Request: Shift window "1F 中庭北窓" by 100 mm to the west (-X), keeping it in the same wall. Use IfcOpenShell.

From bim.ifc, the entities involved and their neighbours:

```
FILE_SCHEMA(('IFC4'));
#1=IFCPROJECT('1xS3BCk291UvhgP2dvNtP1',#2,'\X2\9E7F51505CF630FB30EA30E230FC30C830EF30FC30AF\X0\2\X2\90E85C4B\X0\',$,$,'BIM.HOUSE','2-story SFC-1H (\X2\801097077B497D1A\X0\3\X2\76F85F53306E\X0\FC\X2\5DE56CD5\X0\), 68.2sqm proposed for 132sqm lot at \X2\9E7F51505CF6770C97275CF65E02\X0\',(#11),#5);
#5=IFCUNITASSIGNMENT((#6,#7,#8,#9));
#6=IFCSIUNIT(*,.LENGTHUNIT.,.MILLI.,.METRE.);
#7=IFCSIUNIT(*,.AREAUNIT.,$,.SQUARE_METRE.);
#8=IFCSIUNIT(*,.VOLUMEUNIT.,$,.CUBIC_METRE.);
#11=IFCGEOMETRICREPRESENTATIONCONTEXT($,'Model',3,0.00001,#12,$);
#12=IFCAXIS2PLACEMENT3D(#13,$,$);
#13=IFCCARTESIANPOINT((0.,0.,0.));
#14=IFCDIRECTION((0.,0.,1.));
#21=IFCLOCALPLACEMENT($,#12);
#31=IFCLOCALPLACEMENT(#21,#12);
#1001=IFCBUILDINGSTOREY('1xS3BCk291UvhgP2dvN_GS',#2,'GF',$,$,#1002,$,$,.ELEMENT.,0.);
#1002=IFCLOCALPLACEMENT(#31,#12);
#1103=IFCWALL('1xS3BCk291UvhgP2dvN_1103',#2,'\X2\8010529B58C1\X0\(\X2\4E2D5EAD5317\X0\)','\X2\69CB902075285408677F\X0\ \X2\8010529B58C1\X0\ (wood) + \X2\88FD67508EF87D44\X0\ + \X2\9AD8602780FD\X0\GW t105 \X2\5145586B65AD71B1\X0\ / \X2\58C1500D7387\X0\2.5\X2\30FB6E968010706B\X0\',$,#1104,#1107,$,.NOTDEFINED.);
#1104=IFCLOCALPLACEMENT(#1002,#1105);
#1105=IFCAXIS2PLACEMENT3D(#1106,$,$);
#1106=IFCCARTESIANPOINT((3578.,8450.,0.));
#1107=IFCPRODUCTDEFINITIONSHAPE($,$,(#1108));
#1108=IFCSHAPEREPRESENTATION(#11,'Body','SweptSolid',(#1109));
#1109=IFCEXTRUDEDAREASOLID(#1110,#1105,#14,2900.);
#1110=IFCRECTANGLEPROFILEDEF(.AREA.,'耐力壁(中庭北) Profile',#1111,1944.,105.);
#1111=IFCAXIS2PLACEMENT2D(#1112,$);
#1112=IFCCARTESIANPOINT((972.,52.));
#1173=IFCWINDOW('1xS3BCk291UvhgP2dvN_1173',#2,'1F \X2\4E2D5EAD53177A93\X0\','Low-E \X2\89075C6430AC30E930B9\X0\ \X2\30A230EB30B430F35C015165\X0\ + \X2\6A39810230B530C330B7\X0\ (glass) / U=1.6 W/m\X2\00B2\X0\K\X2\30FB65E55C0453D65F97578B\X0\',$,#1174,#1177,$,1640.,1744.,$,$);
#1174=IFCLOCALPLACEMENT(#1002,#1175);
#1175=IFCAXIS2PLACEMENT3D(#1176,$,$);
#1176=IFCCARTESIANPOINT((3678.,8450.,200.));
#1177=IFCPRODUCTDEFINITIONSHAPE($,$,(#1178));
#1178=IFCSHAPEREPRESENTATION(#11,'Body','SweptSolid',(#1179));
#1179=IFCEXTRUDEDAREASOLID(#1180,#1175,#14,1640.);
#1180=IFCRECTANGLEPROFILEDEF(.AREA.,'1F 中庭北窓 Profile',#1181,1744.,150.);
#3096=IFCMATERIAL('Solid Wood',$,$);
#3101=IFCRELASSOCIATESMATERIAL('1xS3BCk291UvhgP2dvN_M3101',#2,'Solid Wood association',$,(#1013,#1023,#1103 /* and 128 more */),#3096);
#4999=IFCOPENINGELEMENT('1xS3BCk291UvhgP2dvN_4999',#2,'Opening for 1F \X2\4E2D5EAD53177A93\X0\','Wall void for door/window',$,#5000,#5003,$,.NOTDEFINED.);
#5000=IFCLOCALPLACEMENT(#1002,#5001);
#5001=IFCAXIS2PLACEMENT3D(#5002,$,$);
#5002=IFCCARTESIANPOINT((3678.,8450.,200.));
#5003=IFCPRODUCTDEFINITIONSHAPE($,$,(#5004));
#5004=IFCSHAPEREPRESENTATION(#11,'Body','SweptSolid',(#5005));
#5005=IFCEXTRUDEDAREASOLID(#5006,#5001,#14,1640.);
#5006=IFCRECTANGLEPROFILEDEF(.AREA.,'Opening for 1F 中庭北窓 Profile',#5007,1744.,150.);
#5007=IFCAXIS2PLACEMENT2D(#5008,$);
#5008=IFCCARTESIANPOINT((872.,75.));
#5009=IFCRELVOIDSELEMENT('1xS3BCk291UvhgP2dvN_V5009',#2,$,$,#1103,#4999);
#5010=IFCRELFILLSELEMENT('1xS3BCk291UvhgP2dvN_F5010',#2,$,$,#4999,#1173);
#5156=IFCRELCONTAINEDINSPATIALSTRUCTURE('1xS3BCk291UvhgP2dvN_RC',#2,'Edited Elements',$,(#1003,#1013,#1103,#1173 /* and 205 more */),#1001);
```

```python
import ifcopenshell
import ifcopenshell.api.geometry
import ifcopenshell.util.placement
import ifcopenshell.util.unit

model = ifcopenshell.open("bim.ifc")
unit_scale = ifcopenshell.util.unit.calculate_unit_scale(model)

window = model.by_id(1173)
opening = window.FillsVoids[0].RelatingOpeningElement
wall = opening.VoidsElements[0].RelatingBuildingElement

wall_matrix = ifcopenshell.util.placement.get_local_placement(wall.ObjectPlacement)
shift = wall_matrix[:3, 0] * -0.1 / unit_scale
before = ifcopenshell.util.placement.get_local_placement(window.ObjectPlacement)[:3, 3].copy()

# The window is not placed relative to its opening, so move both.
for product in (opening, window):
    matrix = ifcopenshell.util.placement.get_local_placement(product.ObjectPlacement)
    matrix[:3, 3] += shift
    ifcopenshell.api.geometry.edit_object_placement(model, product=product, matrix=matrix, is_si=False)

after = ifcopenshell.util.placement.get_local_placement(window.ObjectPlacement)[:3, 3]
print("window moved by", (after - before).round(3) + 0.0)

model.write("bim_v2.ifc")
```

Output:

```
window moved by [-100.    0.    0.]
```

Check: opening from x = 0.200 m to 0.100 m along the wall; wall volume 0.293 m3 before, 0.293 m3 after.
